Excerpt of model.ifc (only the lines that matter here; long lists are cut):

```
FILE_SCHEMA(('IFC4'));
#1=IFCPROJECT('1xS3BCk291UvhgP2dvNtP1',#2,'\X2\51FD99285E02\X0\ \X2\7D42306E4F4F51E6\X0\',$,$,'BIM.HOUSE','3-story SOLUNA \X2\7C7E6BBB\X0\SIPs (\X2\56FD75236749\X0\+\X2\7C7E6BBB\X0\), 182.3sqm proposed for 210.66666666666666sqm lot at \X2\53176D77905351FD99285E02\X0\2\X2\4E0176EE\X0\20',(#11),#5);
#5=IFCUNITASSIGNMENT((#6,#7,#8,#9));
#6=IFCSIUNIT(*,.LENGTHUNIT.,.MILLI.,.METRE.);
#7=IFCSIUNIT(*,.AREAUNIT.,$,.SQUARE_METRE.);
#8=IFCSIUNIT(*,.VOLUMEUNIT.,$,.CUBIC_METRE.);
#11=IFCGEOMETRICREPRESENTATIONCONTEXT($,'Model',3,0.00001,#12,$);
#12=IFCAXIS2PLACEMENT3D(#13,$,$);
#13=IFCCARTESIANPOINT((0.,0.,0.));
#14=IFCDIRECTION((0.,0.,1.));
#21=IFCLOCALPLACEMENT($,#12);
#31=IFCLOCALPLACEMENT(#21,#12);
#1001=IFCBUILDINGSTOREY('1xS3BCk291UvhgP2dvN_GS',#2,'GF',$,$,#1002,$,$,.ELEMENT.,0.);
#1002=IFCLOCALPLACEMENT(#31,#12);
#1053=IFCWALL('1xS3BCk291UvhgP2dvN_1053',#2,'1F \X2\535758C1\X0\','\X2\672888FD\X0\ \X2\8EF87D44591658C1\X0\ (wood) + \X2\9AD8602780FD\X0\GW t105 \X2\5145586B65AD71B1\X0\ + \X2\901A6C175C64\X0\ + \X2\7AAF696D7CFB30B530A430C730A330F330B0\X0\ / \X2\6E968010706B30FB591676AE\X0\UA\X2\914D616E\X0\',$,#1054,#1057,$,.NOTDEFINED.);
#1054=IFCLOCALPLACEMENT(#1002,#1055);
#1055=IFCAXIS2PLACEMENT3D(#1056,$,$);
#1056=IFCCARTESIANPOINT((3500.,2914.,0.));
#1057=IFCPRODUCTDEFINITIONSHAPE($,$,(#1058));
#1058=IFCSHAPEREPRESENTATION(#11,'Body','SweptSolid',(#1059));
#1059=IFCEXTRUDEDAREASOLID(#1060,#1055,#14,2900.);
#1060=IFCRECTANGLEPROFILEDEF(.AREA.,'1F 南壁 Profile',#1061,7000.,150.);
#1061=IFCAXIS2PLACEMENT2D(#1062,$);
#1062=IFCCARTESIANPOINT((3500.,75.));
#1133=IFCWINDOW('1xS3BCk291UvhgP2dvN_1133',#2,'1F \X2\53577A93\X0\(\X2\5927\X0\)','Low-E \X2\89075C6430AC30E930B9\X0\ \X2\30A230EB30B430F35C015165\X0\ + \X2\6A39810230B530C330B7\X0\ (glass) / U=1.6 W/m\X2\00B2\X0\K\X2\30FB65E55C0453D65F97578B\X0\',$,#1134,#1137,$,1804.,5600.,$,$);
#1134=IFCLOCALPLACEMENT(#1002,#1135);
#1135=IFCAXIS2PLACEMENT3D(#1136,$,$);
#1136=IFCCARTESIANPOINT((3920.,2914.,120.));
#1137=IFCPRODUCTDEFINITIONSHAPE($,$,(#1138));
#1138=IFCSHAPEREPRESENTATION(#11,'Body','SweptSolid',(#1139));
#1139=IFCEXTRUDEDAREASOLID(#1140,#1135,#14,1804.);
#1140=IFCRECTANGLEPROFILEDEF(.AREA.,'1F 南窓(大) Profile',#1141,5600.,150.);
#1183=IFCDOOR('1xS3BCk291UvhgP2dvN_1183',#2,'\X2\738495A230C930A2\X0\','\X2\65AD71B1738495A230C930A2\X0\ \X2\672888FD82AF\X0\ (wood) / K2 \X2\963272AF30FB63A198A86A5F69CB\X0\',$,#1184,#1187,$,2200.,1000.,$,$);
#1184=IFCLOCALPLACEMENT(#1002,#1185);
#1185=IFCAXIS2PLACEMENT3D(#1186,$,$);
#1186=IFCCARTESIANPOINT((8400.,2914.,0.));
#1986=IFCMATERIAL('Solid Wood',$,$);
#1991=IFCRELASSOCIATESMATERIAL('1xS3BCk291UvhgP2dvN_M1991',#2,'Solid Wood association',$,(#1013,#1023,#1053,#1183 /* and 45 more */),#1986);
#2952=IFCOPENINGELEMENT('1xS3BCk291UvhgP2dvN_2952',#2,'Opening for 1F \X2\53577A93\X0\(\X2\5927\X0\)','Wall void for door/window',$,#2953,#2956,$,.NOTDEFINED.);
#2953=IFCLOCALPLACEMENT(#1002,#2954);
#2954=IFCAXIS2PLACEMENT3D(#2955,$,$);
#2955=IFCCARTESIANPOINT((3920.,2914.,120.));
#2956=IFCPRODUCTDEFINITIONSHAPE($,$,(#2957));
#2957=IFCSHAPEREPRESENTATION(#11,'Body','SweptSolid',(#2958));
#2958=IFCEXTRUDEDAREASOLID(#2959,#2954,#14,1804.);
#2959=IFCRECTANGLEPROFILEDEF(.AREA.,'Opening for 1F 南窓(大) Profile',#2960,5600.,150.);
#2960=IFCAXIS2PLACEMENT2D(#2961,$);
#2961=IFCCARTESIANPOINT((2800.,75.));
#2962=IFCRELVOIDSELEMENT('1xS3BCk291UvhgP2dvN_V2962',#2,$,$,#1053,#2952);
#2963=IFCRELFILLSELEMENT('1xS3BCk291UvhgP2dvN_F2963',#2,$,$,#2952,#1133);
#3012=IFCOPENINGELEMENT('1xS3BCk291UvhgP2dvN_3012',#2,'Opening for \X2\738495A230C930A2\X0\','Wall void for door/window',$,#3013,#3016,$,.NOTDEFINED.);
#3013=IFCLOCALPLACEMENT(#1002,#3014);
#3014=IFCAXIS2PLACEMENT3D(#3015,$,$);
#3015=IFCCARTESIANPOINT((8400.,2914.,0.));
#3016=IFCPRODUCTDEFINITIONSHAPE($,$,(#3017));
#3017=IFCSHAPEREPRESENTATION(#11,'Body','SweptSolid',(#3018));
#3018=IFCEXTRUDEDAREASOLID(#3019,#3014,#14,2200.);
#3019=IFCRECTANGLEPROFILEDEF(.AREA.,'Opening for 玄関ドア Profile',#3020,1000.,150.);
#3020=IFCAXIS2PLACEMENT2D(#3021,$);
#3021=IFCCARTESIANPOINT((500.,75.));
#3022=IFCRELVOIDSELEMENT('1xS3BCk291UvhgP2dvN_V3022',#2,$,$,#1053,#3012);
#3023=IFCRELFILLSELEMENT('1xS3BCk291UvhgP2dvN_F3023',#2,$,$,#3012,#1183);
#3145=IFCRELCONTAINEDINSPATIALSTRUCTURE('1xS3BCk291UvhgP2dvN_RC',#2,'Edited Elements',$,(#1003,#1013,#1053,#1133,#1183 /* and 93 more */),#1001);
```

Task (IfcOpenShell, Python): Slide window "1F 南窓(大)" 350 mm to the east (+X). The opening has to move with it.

```python
import ifcopenshell
import ifcopenshell.api.geometry
import ifcopenshell.util.placement
import ifcopenshell.util.unit

model = ifcopenshell.open("model.ifc")
unit_scale = ifcopenshell.util.unit.calculate_unit_scale(model)

window = model.by_guid("1xS3BCk291UvhgP2dvN_1133")
opening = window.FillsVoids[0].RelatingOpeningElement
wall = opening.VoidsElements[0].RelatingBuildingElement

wall_matrix = ifcopenshell.util.placement.get_local_placement(wall.ObjectPlacement)
shift = wall_matrix[:3, 0] * 0.35 / unit_scale
before = ifcopenshell.util.placement.get_local_placement(window.ObjectPlacement)[:3, 3].copy()

# The window is not placed relative to its opening, so move both.
for product in (opening, window):
    matrix = ifcopenshell.util.placement.get_local_placement(product.ObjectPlacement)
    matrix[:3, 3] += shift
    ifcopenshell.api.geometry.edit_object_placement(model, product=product, matrix=matrix, is_si=False)

after = ifcopenshell.util.placement.get_local_placement(window.ObjectPlacement)[:3, 3]
print("window moved by", (after - before).round(3) + 0.0)

model.write("model_v2.ifc")
```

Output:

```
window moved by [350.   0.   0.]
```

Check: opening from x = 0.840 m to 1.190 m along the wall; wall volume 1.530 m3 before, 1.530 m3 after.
